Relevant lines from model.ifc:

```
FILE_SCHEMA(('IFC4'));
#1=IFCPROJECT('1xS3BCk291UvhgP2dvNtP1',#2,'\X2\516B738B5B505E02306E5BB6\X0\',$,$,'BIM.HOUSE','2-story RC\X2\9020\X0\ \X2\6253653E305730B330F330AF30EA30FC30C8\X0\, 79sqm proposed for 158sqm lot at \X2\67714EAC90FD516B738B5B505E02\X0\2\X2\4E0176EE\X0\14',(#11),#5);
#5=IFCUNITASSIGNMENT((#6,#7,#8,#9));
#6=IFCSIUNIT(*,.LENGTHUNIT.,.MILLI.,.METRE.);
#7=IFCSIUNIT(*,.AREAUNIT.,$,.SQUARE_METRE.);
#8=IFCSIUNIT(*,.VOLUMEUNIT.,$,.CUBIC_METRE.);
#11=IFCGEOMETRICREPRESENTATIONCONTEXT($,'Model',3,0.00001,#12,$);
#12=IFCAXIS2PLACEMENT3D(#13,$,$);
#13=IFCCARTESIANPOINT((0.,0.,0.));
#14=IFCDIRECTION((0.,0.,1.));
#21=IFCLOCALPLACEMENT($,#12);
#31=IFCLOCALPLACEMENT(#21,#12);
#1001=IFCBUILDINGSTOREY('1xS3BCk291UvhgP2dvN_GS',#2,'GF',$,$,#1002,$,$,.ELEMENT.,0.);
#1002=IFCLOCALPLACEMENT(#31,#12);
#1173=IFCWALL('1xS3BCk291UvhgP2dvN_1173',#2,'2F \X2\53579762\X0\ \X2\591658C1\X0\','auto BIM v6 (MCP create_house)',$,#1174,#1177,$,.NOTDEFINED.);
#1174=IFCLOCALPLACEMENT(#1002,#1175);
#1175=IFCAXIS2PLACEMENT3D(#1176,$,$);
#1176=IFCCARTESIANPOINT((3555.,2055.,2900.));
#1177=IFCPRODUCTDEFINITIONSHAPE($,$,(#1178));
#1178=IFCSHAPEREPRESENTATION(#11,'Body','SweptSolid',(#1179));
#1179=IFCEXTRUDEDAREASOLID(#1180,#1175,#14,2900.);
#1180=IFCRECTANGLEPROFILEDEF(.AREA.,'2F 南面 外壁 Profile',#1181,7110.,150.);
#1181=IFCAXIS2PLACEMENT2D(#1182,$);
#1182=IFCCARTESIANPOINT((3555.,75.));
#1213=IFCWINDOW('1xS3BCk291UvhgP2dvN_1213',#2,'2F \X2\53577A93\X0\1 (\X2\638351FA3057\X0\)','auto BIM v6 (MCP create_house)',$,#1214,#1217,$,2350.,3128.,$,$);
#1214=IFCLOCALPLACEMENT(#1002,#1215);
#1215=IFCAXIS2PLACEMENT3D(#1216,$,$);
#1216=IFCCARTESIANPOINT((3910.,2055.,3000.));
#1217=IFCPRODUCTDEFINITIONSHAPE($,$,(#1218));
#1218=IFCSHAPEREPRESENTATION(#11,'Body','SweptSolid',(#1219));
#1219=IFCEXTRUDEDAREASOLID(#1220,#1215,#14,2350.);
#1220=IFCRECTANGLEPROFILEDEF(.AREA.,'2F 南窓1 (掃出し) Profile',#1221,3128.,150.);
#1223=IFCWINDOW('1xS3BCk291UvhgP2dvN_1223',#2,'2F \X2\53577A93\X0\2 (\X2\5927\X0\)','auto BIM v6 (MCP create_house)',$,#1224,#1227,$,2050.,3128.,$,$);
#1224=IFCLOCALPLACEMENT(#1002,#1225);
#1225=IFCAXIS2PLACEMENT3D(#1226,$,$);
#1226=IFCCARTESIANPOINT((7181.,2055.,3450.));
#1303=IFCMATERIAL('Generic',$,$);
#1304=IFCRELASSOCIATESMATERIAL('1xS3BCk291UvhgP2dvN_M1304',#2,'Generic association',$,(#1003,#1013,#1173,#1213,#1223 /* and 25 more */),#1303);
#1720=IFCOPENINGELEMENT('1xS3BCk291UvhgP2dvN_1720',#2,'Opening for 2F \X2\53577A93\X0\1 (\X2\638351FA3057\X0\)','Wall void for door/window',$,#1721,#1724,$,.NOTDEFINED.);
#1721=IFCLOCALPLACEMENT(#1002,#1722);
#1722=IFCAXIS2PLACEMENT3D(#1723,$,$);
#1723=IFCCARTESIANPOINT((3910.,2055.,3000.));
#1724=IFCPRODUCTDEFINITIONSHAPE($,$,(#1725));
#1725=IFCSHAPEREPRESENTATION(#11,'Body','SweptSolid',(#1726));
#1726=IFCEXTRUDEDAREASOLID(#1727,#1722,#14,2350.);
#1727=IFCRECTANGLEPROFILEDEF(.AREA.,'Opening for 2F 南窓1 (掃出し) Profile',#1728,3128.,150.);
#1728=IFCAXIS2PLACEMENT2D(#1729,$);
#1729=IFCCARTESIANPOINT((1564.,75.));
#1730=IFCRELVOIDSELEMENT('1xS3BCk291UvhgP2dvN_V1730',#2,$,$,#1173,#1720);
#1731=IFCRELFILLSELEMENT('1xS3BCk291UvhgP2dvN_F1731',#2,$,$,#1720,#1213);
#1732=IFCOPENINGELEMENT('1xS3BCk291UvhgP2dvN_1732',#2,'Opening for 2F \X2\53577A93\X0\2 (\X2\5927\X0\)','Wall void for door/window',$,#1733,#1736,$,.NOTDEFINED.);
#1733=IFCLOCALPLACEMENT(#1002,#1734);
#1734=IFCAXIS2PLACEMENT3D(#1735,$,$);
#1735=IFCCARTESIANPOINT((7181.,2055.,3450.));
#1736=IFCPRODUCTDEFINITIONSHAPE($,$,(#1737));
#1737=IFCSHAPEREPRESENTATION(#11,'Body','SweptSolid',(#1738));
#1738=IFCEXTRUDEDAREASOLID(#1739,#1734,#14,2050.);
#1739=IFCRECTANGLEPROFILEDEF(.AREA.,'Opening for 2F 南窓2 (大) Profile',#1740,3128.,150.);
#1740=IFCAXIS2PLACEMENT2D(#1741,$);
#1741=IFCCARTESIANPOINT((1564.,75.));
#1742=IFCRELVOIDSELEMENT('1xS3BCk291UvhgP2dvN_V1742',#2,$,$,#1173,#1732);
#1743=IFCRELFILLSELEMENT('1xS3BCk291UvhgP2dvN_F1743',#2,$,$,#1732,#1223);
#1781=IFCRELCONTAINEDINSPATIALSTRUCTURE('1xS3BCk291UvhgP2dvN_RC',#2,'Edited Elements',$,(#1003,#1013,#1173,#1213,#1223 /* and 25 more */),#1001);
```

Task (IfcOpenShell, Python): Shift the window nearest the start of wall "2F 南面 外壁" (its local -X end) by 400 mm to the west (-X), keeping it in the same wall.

```python
import ifcopenshell
import ifcopenshell.api.geometry
import ifcopenshell.util.placement
import ifcopenshell.util.unit

model = ifcopenshell.open("model.ifc")
unit_scale = ifcopenshell.util.unit.calculate_unit_scale(model)

window = model.by_id(1213)
opening = window.FillsVoids[0].RelatingOpeningElement
wall = opening.VoidsElements[0].RelatingBuildingElement

wall_matrix = ifcopenshell.util.placement.get_local_placement(wall.ObjectPlacement)
shift = wall_matrix[:3, 0] * -0.4 / unit_scale
before = ifcopenshell.util.placement.get_local_placement(window.ObjectPlacement)[:3, 3].copy()

# The window is not placed relative to its opening, so move both.
for product in (opening, window):
    matrix = ifcopenshell.util.placement.get_local_placement(product.ObjectPlacement)
    matrix[:3, 3] += shift
    ifcopenshell.api.geometry.edit_object_placement(model, product=product, matrix=matrix, is_si=False)

after = ifcopenshell.util.placement.get_local_placement(window.ObjectPlacement)[:3, 3]
print("window moved by", (after - before).round(3) + 0.0)

model.write("model_rev.ifc")
```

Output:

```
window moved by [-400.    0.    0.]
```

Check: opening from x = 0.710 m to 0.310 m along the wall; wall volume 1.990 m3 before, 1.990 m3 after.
